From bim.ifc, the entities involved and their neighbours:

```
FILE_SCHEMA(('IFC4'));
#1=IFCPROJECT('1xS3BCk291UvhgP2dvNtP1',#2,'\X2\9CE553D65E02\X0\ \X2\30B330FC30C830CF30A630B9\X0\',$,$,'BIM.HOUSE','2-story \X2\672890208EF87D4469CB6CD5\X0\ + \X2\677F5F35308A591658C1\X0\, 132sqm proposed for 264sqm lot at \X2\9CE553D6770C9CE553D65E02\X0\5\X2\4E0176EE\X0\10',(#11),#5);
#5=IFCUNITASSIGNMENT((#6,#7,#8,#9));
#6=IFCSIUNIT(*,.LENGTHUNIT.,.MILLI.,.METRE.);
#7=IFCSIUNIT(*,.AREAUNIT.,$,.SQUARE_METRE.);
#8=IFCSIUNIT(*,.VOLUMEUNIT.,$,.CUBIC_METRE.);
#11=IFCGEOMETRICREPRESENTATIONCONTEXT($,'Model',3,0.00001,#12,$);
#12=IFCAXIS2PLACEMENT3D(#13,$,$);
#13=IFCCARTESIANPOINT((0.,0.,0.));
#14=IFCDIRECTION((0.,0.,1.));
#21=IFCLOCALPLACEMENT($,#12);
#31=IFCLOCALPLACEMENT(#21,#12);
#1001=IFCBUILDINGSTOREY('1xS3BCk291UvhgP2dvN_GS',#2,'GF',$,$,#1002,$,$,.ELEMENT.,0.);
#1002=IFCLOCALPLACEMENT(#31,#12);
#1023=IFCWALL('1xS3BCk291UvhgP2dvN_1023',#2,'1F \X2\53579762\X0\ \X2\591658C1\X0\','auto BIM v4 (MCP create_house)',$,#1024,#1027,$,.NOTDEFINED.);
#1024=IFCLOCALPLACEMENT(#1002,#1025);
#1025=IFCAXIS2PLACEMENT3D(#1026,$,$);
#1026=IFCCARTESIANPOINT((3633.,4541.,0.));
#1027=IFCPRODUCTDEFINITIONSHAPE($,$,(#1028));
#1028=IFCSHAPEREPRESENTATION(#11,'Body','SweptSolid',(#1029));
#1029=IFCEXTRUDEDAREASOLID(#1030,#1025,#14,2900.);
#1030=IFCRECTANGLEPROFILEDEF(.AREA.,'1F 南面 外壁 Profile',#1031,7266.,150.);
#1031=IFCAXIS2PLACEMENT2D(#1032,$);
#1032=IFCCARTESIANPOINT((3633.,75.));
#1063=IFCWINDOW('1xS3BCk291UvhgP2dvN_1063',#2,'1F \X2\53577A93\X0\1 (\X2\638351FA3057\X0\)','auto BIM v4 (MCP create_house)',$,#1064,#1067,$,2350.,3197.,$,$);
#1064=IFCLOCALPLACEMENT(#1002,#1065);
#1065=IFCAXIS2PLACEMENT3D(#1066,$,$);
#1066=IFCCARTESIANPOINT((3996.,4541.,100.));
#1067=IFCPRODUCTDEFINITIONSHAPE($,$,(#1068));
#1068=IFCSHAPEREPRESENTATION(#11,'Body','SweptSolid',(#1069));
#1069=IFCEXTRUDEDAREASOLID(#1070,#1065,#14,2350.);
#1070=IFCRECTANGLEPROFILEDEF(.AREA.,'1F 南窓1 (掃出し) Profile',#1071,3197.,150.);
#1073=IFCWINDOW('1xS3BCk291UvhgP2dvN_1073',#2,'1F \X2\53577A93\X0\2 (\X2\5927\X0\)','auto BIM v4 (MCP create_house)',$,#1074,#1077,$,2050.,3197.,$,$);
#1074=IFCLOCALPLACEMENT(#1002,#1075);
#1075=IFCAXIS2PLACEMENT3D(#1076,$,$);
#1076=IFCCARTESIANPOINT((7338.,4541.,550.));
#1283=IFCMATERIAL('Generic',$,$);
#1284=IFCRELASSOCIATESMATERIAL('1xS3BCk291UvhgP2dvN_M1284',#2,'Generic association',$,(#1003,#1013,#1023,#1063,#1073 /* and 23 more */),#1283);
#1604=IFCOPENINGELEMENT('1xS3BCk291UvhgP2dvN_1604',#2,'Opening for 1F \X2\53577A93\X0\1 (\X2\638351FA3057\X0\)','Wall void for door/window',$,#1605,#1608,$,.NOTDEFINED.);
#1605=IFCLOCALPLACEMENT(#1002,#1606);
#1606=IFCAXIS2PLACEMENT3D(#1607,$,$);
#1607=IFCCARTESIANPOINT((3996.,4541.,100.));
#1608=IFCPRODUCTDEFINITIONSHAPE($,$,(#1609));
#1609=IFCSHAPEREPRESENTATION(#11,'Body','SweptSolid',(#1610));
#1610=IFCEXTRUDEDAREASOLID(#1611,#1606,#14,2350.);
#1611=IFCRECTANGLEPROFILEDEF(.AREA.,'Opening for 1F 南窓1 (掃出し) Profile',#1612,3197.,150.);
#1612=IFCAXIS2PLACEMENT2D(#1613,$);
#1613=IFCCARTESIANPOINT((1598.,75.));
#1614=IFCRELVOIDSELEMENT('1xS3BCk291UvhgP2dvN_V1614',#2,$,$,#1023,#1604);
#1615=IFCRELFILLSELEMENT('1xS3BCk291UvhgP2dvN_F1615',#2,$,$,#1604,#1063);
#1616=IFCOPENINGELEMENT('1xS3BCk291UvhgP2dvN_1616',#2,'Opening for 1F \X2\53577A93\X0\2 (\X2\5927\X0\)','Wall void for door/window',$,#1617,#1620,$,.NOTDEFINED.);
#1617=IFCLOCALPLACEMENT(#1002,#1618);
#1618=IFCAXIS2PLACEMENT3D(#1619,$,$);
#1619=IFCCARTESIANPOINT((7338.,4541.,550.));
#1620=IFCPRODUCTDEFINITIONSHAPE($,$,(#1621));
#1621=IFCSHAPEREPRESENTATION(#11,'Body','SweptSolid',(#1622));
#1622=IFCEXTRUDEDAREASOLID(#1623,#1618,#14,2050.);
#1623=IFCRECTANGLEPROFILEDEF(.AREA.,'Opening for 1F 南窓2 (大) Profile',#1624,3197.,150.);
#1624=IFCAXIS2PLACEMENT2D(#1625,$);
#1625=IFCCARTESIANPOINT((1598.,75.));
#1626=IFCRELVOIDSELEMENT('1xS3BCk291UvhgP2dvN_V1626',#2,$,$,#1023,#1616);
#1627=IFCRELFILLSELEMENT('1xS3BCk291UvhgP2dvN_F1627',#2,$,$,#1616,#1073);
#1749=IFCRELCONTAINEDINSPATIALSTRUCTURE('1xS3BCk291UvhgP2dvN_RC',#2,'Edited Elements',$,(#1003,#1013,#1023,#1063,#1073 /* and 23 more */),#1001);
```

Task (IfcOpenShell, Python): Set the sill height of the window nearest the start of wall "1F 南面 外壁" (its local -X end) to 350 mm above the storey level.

```python
import numpy as np
import ifcopenshell
import ifcopenshell.api.geometry
import ifcopenshell.geom
import ifcopenshell.util.element
import ifcopenshell.util.placement
import ifcopenshell.util.shape
import ifcopenshell.util.unit

model = ifcopenshell.open("bim.ifc")
unit_scale = ifcopenshell.util.unit.calculate_unit_scale(model)

window = model.by_guid("1xS3BCk291UvhgP2dvN_1063")
opening = window.FillsVoids[0].RelatingOpeningElement
storey = ifcopenshell.util.element.get_container(window, ifc_class="IfcBuildingStorey")
level = ifcopenshell.util.placement.get_local_placement(storey.ObjectPlacement)[2, 3]

# The opening's origin need not be at the sill, so measure its lowest point.
shape = ifcopenshell.geom.create_shape(ifcopenshell.geom.settings(), opening)
bottom = ifcopenshell.util.shape.get_shape_bottom_elevation(shape, shape.geometry) / unit_scale
dz = level + 0.35 / unit_scale - bottom

shift = np.array([0.0, 0.0, dz])
# The window is not placed relative to its opening, so move both.
for product in (opening, window):
    matrix = ifcopenshell.util.placement.get_local_placement(product.ObjectPlacement)
    matrix[:3, 3] += shift
    ifcopenshell.api.geometry.edit_object_placement(model, product=product, matrix=matrix, is_si=False)

print(f"moved by {dz * unit_scale:+.3f} m")

model.write("bim_rev.ifc")
```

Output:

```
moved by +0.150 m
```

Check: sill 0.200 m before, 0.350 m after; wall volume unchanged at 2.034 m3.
